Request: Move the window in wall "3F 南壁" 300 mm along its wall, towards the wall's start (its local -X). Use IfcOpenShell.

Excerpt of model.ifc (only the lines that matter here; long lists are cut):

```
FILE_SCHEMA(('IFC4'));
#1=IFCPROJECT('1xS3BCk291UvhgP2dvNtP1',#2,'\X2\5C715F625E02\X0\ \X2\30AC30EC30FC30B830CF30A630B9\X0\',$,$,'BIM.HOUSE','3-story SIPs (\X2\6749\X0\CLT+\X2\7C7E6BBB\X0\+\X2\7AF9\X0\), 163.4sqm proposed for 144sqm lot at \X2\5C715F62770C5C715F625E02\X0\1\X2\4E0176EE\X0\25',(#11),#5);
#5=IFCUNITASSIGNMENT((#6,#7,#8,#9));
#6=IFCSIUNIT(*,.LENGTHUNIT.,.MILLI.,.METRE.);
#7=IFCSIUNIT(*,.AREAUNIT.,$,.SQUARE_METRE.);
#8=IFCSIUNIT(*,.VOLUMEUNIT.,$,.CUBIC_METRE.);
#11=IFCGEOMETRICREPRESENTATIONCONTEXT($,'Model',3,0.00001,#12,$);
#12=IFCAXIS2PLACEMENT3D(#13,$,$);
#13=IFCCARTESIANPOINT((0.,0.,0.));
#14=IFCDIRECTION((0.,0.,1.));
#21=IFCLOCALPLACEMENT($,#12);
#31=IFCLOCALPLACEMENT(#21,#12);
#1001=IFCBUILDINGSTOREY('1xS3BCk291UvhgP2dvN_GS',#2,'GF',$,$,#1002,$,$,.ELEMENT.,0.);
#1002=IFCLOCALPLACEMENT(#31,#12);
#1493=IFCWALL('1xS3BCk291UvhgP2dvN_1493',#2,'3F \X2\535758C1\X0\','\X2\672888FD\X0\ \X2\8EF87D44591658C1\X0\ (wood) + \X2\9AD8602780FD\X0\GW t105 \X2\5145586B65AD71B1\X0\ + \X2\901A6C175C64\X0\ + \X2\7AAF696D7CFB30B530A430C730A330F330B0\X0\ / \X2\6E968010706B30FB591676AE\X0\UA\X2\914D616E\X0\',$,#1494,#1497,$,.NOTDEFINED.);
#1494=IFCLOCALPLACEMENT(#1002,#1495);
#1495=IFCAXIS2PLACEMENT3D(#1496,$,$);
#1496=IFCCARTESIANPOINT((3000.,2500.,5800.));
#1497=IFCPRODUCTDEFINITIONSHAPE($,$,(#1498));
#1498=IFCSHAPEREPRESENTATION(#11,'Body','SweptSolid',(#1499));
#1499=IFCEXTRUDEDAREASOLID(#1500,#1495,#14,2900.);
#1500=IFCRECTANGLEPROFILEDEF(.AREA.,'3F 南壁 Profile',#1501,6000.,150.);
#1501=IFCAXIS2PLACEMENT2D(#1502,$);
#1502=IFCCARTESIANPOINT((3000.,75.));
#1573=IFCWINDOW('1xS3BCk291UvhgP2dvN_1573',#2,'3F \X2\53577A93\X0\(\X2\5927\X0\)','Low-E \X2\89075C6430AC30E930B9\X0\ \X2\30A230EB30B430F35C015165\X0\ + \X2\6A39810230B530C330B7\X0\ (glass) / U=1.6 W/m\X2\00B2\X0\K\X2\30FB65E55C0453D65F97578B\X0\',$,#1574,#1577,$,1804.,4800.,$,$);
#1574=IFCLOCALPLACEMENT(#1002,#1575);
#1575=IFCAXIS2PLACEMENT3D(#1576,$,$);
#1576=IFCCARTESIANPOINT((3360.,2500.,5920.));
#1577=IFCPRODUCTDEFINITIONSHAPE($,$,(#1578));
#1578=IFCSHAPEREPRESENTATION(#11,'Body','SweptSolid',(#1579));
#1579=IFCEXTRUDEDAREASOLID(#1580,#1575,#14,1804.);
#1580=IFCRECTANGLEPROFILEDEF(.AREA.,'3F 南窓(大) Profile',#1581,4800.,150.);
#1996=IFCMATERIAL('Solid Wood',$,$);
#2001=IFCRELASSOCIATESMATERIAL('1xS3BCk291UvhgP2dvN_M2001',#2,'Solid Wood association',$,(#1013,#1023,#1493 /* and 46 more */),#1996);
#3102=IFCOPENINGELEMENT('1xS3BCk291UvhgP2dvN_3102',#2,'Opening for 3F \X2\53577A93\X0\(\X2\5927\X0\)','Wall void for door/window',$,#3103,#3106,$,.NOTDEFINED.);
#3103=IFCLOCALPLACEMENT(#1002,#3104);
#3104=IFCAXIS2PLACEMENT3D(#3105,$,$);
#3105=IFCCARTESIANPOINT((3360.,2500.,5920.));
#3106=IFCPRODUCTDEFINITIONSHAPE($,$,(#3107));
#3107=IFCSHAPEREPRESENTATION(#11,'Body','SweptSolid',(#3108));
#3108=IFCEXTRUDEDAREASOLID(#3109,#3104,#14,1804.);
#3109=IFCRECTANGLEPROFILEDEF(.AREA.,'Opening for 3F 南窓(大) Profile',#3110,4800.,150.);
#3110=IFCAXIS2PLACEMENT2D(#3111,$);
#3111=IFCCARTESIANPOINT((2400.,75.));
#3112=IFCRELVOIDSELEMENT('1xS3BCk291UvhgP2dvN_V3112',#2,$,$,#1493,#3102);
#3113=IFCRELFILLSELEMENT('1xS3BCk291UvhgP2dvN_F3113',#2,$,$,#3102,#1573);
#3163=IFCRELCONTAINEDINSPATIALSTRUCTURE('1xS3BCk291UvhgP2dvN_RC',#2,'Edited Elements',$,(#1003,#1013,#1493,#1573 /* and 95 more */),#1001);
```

```python
import ifcopenshell
import ifcopenshell.api.geometry
import ifcopenshell.util.placement
import ifcopenshell.util.unit

model = ifcopenshell.open("model.ifc")
unit_scale = ifcopenshell.util.unit.calculate_unit_scale(model)

window = model.by_guid("1xS3BCk291UvhgP2dvN_1573")
opening = window.FillsVoids[0].RelatingOpeningElement
wall = opening.VoidsElements[0].RelatingBuildingElement

wall_matrix = ifcopenshell.util.placement.get_local_placement(wall.ObjectPlacement)
shift = wall_matrix[:3, 0] * -0.3 / unit_scale
before = ifcopenshell.util.placement.get_local_placement(window.ObjectPlacement)[:3, 3].copy()

# The window is not placed relative to its opening, so move both.
for product in (opening, window):
    matrix = ifcopenshell.util.placement.get_local_placement(product.ObjectPlacement)
    matrix[:3, 3] += shift
    ifcopenshell.api.geometry.edit_object_placement(model, product=product, matrix=matrix, is_si=False)

after = ifcopenshell.util.placement.get_local_placement(window.ObjectPlacement)[:3, 3]
print("window moved by", (after - before).round(3) + 0.0)

model.write("model_v2.ifc")
```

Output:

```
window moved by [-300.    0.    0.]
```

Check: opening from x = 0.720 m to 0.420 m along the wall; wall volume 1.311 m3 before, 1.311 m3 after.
